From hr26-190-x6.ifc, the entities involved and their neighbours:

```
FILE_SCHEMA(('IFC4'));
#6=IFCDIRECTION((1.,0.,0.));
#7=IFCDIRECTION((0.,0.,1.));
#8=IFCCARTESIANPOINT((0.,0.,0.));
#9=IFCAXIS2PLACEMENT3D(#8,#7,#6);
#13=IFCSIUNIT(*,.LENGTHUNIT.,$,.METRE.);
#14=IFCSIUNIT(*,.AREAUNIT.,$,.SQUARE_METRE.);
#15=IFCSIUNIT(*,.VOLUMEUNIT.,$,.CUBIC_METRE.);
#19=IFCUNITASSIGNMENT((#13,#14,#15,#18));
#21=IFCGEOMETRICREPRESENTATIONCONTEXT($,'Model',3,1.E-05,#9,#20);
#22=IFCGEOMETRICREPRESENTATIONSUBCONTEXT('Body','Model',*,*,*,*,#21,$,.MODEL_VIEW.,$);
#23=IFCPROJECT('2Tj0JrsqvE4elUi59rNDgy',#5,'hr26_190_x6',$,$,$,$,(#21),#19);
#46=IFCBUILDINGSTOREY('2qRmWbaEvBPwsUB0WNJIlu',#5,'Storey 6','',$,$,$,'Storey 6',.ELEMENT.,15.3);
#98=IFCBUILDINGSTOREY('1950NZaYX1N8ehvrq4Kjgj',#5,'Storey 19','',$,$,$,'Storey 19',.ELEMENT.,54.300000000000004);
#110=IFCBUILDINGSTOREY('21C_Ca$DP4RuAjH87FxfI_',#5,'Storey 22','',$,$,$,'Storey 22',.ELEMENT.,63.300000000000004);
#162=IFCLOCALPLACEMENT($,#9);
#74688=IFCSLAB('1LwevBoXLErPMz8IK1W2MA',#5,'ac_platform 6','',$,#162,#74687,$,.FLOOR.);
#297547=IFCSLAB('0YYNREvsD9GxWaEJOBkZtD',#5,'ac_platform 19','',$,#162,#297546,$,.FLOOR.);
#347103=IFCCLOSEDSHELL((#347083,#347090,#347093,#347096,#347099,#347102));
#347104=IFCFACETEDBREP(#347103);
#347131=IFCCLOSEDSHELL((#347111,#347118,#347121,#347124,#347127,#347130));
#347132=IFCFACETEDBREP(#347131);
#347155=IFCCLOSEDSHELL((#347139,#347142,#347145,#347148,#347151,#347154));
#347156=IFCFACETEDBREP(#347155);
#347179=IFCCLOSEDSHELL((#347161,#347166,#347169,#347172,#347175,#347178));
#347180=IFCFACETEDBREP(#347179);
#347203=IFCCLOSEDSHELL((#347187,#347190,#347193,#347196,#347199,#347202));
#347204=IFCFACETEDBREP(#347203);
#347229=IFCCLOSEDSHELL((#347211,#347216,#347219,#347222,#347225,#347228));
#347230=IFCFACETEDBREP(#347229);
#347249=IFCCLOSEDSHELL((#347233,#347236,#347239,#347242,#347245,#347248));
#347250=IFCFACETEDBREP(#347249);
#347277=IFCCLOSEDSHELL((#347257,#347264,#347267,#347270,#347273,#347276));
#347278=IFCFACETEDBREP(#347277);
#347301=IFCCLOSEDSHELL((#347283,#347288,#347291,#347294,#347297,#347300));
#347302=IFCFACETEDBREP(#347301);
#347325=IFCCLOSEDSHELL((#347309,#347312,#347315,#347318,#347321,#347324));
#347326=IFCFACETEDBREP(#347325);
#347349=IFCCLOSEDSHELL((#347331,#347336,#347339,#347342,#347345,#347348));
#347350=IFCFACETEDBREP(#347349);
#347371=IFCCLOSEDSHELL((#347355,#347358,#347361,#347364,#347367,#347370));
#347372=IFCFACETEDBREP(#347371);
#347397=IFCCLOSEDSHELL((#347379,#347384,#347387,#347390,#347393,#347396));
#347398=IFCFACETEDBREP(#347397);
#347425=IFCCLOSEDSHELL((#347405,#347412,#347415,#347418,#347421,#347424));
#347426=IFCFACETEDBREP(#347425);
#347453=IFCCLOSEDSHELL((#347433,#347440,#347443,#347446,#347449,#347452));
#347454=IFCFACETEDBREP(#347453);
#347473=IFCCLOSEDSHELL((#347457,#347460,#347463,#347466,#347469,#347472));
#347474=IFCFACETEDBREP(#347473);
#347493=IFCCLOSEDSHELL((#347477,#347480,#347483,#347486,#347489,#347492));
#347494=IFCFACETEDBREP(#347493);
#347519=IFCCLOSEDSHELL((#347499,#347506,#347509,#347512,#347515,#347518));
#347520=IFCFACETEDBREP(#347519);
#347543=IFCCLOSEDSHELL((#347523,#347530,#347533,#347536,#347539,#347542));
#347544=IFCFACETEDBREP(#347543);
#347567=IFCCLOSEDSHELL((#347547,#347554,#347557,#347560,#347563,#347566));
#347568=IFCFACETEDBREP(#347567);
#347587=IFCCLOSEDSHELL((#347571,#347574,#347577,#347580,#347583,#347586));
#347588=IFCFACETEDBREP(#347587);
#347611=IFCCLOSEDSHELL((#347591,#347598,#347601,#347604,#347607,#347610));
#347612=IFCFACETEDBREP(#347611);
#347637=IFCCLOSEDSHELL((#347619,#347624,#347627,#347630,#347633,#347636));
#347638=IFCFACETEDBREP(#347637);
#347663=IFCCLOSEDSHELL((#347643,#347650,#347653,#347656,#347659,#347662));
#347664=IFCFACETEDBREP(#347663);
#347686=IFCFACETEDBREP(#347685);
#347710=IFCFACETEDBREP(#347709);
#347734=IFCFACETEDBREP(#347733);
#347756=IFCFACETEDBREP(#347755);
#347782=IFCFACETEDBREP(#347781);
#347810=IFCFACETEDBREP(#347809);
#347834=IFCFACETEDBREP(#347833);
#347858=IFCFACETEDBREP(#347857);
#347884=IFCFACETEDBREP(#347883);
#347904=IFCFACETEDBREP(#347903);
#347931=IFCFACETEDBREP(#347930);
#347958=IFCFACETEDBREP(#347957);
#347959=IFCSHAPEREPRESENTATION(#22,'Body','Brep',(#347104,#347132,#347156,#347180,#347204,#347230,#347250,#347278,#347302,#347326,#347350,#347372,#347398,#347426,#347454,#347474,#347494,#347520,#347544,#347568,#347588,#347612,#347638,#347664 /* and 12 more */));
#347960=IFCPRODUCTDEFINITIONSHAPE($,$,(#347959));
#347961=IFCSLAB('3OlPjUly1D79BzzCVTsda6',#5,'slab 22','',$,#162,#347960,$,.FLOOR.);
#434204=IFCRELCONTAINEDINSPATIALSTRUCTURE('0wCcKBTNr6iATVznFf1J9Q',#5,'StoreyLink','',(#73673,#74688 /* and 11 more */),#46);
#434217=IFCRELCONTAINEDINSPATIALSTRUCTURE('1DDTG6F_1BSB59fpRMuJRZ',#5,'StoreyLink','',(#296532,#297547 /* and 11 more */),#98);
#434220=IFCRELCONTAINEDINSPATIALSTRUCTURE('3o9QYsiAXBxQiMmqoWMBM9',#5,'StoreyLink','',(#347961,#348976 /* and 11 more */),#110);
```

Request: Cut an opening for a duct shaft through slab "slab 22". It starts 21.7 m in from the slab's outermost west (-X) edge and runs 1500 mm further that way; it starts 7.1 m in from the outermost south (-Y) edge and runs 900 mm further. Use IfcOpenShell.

```python
import numpy as np
import ifcopenshell
import ifcopenshell.api.feature
import ifcopenshell.api.geometry
import ifcopenshell.api.root
import ifcopenshell.geom
import ifcopenshell.util.placement
import ifcopenshell.util.representation
import ifcopenshell.util.shape
import ifcopenshell.util.unit

model = ifcopenshell.open("hr26-190-x6.ifc")
unit_scale = ifcopenshell.util.unit.calculate_unit_scale(model)
settings = ifcopenshell.geom.settings()


def volume(element):
    """Net volume in cubic metres, openings subtracted."""
    shape = ifcopenshell.geom.create_shape(settings, element)
    return ifcopenshell.util.shape.get_volume(shape.geometry)


slab = model.by_guid("3OlPjUly1D79BzzCVTsda6")
before = volume(slab)

# Extent in the slab's own axes, in metres. The edges named are its -X and -Y sides.
slab_shape = ifcopenshell.geom.create_shape(settings, slab)
vertices = ifcopenshell.util.shape.get_vertices(slab_shape.geometry)
x_min, y_min, bottom = vertices.min(axis=0)
top = vertices[:, 2].max()

opening = ifcopenshell.api.root.create_entity(model, ifc_class="IfcOpeningElement", name="Duct shaft opening", predefined_type="OPENING")
context = ifcopenshell.util.representation.get_context(model, "Model", "Body", "MODEL_VIEW")
width, depth = 1.5, 0.9
outline = [(0.0, 0.0), (width, 0.0), (width, depth), (0.0, depth), (0.0, 0.0)]
# Overshoot both faces by 50 mm so the cut is clean.
shape = ifcopenshell.api.geometry.add_slab_representation(
    model, context=context, depth=top - bottom + 0.1, polyline=outline
)
ifcopenshell.api.geometry.assign_representation(model, product=opening, representation=shape)

matrix = ifcopenshell.util.placement.get_local_placement(slab.ObjectPlacement)
matrix[:, 3] = matrix @ np.append(np.array([x_min + 21.7, y_min + 7.1, bottom - 0.05]) / unit_scale, 1.0)
ifcopenshell.api.geometry.edit_object_placement(model, product=opening, matrix=matrix, is_si=False)
ifcopenshell.api.feature.add_feature(model, feature=opening, element=slab)

after = volume(slab)

print(f"slab volume {before:.3f} -> {after:.3f} m3")

model.write("hr26-190-x6-out.ifc")
```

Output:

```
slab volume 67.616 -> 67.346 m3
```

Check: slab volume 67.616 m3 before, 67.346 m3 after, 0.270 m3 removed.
